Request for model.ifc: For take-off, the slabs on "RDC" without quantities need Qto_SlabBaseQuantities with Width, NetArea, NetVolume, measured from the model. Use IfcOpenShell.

First a look at what the model holds.

```python
import ifcopenshell
import ifcopenshell.util.element
import ifcopenshell.util.unit

model = ifcopenshell.open("model.ifc")
print(model.schema)
for unit_type in ("LENGTHUNIT", "AREAUNIT", "VOLUMEUNIT"):
    print(unit_type, ifcopenshell.util.unit.calculate_unit_scale(model, unit_type))
storey = next(s for s in model.by_type("IfcBuildingStorey") if s.Name == "RDC")
slabs = [e for e in ifcopenshell.util.element.get_decomposition(storey) if e.is_a("IfcSlab")]
for e in sorted(slabs, key=lambda e: e.id()):
    print(e.id(), e.is_a(), e.Name, list(ifcopenshell.util.element.get_psets(e, qtos_only=True)), sep=" | ")
```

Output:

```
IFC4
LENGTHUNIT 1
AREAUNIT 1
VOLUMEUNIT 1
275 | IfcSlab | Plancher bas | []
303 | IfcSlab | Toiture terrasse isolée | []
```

```python
import ifcopenshell
import ifcopenshell.api.pset
import ifcopenshell.geom
import ifcopenshell.util.element
import ifcopenshell.util.shape
import ifcopenshell.util.unit

model = ifcopenshell.open("model.ifc")
unit_scale = ifcopenshell.util.unit.calculate_unit_scale(model)
area_scale = ifcopenshell.util.unit.calculate_unit_scale(model, "AREAUNIT")
volume_scale = ifcopenshell.util.unit.calculate_unit_scale(model, "VOLUMEUNIT")
settings = ifcopenshell.geom.settings()

storey = next(s for s in model.by_type("IfcBuildingStorey") if s.Name == "RDC")
slabs = [e for e in ifcopenshell.util.element.get_decomposition(storey) if e.is_a("IfcSlab")]

for e in sorted(slabs, key=lambda e: e.id()):
    if ifcopenshell.util.element.get_psets(e, qtos_only=True, should_inherit=False):
        continue
    # Geometry comes back in metres, in the element's own axes.
    shape = ifcopenshell.geom.create_shape(settings, e)
    values = {
        "Width": ifcopenshell.util.shape.get_z(shape.geometry) / unit_scale,
        "NetArea": ifcopenshell.util.shape.get_footprint_area(shape.geometry) / area_scale,
        "NetVolume": ifcopenshell.util.shape.get_volume(shape.geometry) / volume_scale,
    }
    qto = ifcopenshell.api.pset.add_qto(model, product=e, name="Qto_SlabBaseQuantities")
    ifcopenshell.api.pset.edit_qto(model, qto=qto, properties=values)
    print(e.id(), {k: round(v, 3) for k, v in values.items()})

model.write("model_v2.ifc")
```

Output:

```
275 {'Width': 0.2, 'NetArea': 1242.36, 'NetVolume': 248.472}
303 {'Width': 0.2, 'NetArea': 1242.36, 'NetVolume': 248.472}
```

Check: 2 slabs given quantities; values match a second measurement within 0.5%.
